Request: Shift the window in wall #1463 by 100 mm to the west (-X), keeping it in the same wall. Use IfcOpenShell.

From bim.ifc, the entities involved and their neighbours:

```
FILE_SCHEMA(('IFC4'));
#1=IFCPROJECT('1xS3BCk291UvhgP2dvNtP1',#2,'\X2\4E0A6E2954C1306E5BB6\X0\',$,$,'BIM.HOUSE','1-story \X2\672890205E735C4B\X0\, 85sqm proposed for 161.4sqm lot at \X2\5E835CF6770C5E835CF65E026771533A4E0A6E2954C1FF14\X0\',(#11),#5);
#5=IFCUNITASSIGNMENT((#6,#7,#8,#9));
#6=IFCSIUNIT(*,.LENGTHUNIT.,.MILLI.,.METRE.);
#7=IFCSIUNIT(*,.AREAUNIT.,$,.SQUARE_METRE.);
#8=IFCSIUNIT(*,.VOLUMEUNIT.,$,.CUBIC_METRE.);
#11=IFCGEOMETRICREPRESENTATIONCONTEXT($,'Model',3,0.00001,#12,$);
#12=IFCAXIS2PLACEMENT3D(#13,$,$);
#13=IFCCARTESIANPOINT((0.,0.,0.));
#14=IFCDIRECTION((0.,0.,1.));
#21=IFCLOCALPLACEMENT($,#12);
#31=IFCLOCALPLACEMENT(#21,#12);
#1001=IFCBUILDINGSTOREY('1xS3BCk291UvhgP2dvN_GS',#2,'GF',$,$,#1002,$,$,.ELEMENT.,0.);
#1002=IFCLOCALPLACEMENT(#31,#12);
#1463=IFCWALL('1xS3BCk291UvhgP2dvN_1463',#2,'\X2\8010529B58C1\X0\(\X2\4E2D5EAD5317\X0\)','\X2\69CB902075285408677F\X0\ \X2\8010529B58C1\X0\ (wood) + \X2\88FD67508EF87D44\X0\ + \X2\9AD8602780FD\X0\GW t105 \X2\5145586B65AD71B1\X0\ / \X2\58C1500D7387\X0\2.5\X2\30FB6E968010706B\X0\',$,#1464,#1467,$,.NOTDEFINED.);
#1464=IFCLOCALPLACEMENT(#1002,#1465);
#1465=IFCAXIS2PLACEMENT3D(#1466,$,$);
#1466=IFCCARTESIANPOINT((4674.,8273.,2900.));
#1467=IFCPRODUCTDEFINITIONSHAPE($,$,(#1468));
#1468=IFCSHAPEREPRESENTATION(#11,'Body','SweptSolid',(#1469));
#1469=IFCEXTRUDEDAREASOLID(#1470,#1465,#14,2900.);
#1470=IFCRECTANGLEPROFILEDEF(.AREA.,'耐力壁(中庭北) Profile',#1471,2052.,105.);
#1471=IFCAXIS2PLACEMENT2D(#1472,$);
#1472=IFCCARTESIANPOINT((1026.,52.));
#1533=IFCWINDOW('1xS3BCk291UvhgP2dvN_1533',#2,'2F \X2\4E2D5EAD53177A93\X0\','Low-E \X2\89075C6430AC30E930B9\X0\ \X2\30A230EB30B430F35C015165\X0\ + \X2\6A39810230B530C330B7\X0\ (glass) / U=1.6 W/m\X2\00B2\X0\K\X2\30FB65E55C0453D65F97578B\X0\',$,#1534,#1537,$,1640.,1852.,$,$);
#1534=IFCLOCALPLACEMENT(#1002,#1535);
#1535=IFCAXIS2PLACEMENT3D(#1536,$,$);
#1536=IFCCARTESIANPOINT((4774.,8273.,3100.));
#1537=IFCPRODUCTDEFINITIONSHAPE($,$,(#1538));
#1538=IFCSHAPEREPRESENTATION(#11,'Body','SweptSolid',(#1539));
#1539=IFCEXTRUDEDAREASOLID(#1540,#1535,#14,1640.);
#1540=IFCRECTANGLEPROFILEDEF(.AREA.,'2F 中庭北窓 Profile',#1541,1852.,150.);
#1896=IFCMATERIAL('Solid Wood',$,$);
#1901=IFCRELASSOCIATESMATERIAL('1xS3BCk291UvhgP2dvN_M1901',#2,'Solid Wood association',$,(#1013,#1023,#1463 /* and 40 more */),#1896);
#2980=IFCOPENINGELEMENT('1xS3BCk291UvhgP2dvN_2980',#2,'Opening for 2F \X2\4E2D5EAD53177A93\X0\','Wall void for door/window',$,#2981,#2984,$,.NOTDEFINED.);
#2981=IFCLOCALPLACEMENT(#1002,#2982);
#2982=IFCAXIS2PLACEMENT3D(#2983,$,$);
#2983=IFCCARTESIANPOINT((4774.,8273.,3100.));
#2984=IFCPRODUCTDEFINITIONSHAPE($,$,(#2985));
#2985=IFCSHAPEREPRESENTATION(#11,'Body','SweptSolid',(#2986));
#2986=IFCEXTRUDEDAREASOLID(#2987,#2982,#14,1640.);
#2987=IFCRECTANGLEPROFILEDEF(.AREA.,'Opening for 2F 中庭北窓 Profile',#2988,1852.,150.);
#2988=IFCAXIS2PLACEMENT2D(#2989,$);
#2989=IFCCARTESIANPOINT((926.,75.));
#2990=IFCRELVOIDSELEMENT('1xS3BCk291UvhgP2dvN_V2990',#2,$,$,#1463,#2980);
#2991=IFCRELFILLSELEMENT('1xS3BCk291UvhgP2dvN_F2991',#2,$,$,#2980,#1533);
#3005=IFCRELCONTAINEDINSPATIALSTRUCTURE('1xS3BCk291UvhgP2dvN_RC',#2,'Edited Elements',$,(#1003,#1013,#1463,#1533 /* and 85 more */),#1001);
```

```python
import ifcopenshell
import ifcopenshell.api.geometry
import ifcopenshell.util.placement

model = ifcopenshell.open("bim.ifc")

window = model.by_guid("1xS3BCk291UvhgP2dvN_1533")
opening = window.FillsVoids[0].RelatingOpeningElement
wall = opening.VoidsElements[0].RelatingBuildingElement

wall_matrix = ifcopenshell.util.placement.get_local_placement(wall.ObjectPlacement)
shift = wall_matrix[:3, 0] * -100.0
before = ifcopenshell.util.placement.get_local_placement(window.ObjectPlacement)[:3, 3].copy()

# The window is not placed relative to its opening, so move both.
for product in (opening, window):
    matrix = ifcopenshell.util.placement.get_local_placement(product.ObjectPlacement)
    matrix[:3, 3] += shift
    ifcopenshell.api.geometry.edit_object_placement(model, product=product, matrix=matrix, is_si=False)

after = ifcopenshell.util.placement.get_local_placement(window.ObjectPlacement)[:3, 3]
print("window moved by", (after - before).round(3) + 0.0)

model.write("bim_updated.ifc")
```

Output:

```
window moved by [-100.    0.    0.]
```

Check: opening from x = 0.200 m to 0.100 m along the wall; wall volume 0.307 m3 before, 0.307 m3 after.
